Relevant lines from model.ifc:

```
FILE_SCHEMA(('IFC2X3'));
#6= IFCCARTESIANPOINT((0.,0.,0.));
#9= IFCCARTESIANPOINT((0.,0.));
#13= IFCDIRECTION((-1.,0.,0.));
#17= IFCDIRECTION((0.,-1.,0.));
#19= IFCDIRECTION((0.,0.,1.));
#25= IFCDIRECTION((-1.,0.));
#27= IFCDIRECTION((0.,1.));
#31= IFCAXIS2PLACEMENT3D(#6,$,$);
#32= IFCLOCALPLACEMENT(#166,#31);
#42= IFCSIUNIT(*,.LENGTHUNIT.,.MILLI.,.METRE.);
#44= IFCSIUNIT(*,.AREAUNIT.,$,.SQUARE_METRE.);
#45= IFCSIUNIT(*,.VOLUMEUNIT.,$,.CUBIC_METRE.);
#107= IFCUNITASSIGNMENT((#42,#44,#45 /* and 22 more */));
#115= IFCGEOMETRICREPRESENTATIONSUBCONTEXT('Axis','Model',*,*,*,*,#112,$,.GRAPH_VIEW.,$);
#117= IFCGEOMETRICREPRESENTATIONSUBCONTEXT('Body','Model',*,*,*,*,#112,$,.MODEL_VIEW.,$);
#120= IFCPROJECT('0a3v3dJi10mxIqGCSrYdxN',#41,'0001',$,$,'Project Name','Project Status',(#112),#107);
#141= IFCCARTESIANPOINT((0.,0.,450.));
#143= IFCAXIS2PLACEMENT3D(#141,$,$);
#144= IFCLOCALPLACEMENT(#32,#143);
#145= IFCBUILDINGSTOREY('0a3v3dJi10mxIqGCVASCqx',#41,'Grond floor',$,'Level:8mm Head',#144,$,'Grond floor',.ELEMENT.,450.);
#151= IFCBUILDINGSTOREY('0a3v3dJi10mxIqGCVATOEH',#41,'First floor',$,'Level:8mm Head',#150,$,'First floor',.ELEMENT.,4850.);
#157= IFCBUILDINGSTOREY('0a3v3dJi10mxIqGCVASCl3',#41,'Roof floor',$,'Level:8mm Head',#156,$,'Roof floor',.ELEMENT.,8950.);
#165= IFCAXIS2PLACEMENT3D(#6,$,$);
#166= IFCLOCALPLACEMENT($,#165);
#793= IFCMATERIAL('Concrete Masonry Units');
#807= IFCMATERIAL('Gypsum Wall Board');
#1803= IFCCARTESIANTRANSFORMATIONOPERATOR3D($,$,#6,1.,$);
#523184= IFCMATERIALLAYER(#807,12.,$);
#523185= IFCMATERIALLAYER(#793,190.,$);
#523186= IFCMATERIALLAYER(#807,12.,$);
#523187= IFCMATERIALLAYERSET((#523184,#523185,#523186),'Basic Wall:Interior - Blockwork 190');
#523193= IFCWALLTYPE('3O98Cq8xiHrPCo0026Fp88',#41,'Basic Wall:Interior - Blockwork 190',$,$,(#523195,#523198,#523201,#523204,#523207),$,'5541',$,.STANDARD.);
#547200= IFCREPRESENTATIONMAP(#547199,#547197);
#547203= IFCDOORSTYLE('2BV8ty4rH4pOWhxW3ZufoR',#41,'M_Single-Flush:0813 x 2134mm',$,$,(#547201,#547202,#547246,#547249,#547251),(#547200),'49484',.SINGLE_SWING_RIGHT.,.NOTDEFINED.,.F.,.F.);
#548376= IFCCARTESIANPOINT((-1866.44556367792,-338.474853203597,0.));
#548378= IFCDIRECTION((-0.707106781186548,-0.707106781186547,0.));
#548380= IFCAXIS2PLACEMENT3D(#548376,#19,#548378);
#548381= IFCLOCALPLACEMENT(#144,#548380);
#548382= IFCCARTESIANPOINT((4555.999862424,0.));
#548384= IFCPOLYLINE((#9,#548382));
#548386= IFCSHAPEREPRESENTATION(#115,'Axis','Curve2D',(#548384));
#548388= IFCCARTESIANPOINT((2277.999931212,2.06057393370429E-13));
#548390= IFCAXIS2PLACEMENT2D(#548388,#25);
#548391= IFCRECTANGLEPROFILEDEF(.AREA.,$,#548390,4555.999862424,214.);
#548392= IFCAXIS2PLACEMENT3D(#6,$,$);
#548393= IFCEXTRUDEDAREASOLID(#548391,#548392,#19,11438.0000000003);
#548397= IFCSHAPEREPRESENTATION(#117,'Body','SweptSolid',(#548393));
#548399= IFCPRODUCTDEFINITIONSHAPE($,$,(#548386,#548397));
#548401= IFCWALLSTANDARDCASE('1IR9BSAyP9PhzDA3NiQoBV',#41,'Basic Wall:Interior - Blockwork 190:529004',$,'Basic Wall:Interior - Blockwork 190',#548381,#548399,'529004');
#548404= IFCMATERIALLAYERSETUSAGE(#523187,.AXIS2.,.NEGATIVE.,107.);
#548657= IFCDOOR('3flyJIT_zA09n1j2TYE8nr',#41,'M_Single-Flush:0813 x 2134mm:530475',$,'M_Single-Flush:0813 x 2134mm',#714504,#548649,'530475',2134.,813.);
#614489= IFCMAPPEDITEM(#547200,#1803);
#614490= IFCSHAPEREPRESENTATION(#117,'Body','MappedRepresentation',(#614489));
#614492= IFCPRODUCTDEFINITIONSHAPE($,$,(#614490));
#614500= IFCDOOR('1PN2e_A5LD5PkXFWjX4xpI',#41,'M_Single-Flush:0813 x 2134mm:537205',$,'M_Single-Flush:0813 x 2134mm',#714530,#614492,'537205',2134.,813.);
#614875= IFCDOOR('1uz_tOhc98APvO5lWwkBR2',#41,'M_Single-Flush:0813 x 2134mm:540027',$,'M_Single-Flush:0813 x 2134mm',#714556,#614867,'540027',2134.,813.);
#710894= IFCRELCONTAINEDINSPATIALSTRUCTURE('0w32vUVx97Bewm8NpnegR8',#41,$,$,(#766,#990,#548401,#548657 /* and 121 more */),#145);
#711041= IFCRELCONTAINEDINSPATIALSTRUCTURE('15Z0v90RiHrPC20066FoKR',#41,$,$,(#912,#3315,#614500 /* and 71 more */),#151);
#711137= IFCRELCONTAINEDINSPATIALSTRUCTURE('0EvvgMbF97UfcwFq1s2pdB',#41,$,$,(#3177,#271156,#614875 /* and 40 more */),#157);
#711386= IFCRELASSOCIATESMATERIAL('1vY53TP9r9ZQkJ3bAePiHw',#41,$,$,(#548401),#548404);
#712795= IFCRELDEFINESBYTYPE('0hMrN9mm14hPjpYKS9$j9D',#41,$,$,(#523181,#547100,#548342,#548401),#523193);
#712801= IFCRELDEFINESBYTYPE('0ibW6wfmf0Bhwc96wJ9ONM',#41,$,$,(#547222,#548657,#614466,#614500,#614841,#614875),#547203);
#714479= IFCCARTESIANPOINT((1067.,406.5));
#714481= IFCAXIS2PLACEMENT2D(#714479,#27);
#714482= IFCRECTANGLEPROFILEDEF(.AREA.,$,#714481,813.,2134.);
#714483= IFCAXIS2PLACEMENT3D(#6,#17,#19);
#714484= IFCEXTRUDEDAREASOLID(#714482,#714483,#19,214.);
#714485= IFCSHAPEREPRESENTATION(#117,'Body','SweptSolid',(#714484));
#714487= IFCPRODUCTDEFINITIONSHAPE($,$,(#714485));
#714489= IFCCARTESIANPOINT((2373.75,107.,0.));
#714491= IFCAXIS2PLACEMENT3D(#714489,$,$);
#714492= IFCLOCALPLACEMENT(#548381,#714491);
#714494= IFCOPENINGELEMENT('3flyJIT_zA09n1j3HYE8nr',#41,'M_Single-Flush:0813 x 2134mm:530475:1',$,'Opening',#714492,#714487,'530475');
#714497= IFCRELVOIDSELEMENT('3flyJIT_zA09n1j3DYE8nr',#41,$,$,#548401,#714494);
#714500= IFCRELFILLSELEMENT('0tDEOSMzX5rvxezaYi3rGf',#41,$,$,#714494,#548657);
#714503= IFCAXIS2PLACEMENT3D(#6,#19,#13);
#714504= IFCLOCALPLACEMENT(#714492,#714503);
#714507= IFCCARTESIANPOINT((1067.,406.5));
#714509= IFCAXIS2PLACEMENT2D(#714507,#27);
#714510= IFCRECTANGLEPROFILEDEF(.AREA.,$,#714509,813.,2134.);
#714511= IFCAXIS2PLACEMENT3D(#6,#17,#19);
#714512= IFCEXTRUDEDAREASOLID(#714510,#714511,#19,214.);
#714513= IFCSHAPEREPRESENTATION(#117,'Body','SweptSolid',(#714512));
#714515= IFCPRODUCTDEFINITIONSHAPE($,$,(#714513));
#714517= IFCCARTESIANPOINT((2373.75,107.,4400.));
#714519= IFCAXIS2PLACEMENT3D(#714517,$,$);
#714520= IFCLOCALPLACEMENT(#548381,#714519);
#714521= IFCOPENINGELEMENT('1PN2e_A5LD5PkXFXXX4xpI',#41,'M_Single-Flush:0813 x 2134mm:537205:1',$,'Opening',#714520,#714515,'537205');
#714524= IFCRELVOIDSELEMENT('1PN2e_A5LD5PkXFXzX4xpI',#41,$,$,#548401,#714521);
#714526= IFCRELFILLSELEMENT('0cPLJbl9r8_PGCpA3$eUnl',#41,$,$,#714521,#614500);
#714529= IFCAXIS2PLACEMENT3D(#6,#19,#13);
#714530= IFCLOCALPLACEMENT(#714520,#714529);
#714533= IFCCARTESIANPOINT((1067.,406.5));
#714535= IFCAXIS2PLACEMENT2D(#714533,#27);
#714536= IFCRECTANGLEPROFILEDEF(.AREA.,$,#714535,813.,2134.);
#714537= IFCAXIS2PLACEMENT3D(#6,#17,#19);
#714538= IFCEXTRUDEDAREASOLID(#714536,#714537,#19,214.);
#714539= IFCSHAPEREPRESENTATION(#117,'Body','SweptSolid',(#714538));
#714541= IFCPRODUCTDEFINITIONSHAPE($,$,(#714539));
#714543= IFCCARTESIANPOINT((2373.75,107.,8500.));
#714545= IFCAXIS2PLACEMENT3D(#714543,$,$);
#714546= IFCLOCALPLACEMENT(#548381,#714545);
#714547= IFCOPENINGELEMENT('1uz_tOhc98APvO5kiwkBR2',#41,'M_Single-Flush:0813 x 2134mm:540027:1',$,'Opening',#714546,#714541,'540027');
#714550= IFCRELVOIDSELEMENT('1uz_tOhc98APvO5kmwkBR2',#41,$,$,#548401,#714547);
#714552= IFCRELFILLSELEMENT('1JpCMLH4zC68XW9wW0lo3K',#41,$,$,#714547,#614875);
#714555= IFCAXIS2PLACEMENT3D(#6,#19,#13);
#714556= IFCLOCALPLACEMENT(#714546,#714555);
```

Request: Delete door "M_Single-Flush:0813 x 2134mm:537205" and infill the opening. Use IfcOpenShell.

```python
import ifcopenshell
import ifcopenshell.api.feature
import ifcopenshell.api.root
import ifcopenshell.geom
import ifcopenshell.util.shape

model = ifcopenshell.open("model.ifc")
settings = ifcopenshell.geom.settings()


def volume(element):
    """Net volume in cubic metres, openings subtracted."""
    shape = ifcopenshell.geom.create_shape(settings, element)
    return ifcopenshell.util.shape.get_volume(shape.geometry)


door = model.by_id(614500)
opening = door.FillsVoids[0].RelatingOpeningElement
wall = opening.VoidsElements[0].RelatingBuildingElement
before = volume(wall)

ifcopenshell.api.root.remove_product(model, product=door)
ifcopenshell.api.feature.remove_feature(model, feature=opening)

after = volume(wall)

print(f"wall volume {before:.3f} -> {after:.3f} m3")

model.write("model_updated.ifc")
```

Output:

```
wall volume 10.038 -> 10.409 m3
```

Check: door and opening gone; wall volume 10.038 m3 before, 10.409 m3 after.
